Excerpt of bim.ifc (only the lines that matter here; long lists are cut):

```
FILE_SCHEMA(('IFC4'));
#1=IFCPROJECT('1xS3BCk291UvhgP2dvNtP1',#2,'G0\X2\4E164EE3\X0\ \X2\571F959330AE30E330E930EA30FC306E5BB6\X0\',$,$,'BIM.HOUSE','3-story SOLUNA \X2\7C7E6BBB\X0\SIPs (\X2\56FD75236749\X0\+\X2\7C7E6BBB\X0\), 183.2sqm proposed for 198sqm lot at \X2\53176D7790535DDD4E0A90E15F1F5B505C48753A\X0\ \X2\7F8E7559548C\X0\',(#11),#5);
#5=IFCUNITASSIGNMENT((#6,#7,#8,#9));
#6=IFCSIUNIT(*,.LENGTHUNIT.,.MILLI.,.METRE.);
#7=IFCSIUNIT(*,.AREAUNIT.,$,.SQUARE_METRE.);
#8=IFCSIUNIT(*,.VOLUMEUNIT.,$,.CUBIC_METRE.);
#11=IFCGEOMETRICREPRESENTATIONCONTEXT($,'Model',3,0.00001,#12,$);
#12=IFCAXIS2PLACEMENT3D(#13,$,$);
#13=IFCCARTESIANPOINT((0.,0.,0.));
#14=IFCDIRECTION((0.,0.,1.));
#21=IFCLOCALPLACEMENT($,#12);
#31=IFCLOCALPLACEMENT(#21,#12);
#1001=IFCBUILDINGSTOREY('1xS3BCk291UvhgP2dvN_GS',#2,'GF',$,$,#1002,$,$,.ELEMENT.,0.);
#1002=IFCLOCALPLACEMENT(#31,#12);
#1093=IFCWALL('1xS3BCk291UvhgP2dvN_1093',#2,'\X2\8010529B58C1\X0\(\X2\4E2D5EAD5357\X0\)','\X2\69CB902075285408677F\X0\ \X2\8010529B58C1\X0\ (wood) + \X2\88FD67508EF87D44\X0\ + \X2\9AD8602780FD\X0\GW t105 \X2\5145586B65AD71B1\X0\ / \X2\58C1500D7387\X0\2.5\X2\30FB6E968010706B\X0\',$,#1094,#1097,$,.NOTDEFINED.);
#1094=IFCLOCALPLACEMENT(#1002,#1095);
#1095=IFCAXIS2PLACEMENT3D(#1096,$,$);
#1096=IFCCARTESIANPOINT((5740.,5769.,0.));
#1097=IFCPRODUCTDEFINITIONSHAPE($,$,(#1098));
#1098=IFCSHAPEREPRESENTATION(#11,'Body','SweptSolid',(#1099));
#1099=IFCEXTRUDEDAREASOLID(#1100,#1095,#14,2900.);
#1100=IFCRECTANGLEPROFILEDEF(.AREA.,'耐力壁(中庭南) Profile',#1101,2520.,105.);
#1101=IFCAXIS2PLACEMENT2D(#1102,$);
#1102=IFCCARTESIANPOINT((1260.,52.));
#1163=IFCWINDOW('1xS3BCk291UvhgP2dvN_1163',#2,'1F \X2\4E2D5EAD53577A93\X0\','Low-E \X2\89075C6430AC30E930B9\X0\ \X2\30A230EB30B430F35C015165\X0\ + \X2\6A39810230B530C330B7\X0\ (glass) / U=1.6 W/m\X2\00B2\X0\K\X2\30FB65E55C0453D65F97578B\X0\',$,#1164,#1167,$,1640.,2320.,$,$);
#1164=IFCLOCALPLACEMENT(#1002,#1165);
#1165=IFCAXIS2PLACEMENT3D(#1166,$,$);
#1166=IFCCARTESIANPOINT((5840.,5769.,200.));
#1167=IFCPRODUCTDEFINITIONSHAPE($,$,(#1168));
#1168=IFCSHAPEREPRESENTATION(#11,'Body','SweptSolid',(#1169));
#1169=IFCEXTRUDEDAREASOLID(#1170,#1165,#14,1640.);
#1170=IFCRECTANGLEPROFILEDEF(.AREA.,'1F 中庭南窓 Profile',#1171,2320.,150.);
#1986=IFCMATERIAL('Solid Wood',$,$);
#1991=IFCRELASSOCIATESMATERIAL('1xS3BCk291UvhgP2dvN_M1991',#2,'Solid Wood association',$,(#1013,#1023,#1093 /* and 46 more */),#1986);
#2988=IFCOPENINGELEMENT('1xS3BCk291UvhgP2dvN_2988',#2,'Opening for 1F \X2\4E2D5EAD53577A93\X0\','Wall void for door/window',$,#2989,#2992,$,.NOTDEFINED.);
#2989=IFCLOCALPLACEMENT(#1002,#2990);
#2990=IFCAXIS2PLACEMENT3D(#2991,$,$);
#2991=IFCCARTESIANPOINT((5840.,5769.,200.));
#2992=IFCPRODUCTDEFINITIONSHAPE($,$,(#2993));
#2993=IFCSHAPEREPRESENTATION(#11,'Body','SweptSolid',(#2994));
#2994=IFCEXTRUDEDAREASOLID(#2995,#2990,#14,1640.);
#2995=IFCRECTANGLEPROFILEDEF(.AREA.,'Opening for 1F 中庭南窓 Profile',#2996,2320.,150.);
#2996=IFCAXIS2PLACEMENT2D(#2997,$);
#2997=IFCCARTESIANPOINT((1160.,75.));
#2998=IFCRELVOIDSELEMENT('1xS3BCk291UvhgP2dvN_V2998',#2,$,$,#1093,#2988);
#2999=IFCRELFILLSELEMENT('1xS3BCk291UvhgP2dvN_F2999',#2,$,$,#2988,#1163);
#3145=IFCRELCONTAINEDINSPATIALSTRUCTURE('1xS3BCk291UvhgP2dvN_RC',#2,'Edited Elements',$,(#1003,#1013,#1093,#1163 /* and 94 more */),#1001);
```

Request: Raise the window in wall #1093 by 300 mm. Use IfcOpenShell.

```python
import numpy as np
import ifcopenshell
import ifcopenshell.api.geometry
import ifcopenshell.util.placement
import ifcopenshell.util.unit

model = ifcopenshell.open("bim.ifc")
unit_scale = ifcopenshell.util.unit.calculate_unit_scale(model)

window = model.by_guid("1xS3BCk291UvhgP2dvN_1163")
opening = window.FillsVoids[0].RelatingOpeningElement
dz = 0.3 / unit_scale

shift = np.array([0.0, 0.0, dz])
# The window is not placed relative to its opening, so move both.
for product in (opening, window):
    matrix = ifcopenshell.util.placement.get_local_placement(product.ObjectPlacement)
    matrix[:3, 3] += shift
    ifcopenshell.api.geometry.edit_object_placement(model, product=product, matrix=matrix, is_si=False)

print(f"moved by {dz * unit_scale:+.3f} m")

model.write("bim_v2.ifc")
```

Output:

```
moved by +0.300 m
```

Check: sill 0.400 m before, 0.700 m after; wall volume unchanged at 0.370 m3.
